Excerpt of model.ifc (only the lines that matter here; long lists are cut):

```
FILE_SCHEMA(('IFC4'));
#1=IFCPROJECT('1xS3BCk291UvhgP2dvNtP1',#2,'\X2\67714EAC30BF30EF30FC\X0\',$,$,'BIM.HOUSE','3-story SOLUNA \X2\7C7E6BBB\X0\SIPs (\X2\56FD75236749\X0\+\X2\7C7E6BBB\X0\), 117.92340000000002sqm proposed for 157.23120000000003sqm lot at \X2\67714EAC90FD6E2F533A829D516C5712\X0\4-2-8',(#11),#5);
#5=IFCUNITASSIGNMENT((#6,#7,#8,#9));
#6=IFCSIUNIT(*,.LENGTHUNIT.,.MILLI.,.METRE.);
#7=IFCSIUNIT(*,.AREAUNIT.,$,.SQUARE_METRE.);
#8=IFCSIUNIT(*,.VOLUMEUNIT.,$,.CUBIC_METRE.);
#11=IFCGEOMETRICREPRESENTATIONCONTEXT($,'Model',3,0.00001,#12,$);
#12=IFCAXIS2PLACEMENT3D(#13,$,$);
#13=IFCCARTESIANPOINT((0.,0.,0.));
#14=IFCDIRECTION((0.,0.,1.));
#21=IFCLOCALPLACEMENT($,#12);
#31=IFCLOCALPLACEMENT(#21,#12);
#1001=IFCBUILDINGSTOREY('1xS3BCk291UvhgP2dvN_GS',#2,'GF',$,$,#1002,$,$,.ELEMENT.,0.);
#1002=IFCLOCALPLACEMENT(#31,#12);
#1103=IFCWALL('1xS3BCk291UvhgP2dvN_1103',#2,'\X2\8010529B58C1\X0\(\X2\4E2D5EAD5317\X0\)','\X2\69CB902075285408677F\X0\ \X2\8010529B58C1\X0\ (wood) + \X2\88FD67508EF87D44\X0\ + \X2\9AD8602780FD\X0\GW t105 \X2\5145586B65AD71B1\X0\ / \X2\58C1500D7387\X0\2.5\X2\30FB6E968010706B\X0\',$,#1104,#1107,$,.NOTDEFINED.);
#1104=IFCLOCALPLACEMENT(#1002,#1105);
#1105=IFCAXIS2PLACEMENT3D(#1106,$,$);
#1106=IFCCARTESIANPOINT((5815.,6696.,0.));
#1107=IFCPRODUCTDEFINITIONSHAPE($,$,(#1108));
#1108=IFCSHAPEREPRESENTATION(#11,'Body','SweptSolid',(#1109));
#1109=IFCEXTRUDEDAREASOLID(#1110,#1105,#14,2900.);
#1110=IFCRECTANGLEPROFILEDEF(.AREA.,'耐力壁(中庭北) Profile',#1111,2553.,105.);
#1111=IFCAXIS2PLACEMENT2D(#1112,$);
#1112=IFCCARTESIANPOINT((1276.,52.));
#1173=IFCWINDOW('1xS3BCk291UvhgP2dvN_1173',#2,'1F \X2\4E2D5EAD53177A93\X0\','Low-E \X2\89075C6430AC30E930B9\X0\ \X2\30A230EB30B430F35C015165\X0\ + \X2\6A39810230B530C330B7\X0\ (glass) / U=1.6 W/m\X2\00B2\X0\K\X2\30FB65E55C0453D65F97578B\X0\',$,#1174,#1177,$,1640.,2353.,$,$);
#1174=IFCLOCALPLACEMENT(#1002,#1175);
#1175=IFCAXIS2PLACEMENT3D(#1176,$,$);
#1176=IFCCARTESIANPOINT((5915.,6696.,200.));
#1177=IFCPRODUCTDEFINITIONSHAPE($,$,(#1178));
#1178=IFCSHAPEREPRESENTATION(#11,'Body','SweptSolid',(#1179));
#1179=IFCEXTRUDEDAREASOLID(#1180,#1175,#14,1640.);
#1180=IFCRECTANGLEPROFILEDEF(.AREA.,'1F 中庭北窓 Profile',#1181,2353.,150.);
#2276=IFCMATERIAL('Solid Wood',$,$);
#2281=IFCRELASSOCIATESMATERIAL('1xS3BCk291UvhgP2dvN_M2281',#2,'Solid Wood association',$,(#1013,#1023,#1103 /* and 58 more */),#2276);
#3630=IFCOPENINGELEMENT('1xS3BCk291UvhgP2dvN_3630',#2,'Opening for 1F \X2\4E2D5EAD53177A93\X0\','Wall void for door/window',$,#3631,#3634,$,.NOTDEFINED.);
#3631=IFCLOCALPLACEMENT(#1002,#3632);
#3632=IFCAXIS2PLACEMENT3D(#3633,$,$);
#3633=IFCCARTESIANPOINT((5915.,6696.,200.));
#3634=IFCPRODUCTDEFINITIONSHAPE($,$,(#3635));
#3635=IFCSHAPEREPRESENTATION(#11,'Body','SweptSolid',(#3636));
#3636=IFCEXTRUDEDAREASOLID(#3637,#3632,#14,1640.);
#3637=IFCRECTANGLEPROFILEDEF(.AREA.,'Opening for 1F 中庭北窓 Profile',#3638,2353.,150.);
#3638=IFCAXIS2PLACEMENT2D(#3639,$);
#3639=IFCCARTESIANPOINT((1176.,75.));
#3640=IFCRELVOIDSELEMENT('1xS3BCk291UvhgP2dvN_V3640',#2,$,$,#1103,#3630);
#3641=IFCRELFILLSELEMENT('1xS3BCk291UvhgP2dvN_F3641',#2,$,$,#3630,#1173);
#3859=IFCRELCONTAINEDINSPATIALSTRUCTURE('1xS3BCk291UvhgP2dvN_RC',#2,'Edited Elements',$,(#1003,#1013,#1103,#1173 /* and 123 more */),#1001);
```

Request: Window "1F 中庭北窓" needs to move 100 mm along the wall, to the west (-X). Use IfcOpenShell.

```python
import ifcopenshell
import ifcopenshell.api.geometry
import ifcopenshell.util.placement

model = ifcopenshell.open("model.ifc")

window = model.by_guid("1xS3BCk291UvhgP2dvN_1173")
opening = window.FillsVoids[0].RelatingOpeningElement
wall = opening.VoidsElements[0].RelatingBuildingElement

wall_matrix = ifcopenshell.util.placement.get_local_placement(wall.ObjectPlacement)
shift = wall_matrix[:3, 0] * -100.0
before = ifcopenshell.util.placement.get_local_placement(window.ObjectPlacement)[:3, 3].copy()

# The window is not placed relative to its opening, so move both.
for product in (opening, window):
    matrix = ifcopenshell.util.placement.get_local_placement(product.ObjectPlacement)
    matrix[:3, 3] += shift
    ifcopenshell.api.geometry.edit_object_placement(model, product=product, matrix=matrix, is_si=False)

after = ifcopenshell.util.placement.get_local_placement(window.ObjectPlacement)[:3, 3]
print("window moved by", (after - before).round(3) + 0.0)

model.write("model_edited.ifc")
```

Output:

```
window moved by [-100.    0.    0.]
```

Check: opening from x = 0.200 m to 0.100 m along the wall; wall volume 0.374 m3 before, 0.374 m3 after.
